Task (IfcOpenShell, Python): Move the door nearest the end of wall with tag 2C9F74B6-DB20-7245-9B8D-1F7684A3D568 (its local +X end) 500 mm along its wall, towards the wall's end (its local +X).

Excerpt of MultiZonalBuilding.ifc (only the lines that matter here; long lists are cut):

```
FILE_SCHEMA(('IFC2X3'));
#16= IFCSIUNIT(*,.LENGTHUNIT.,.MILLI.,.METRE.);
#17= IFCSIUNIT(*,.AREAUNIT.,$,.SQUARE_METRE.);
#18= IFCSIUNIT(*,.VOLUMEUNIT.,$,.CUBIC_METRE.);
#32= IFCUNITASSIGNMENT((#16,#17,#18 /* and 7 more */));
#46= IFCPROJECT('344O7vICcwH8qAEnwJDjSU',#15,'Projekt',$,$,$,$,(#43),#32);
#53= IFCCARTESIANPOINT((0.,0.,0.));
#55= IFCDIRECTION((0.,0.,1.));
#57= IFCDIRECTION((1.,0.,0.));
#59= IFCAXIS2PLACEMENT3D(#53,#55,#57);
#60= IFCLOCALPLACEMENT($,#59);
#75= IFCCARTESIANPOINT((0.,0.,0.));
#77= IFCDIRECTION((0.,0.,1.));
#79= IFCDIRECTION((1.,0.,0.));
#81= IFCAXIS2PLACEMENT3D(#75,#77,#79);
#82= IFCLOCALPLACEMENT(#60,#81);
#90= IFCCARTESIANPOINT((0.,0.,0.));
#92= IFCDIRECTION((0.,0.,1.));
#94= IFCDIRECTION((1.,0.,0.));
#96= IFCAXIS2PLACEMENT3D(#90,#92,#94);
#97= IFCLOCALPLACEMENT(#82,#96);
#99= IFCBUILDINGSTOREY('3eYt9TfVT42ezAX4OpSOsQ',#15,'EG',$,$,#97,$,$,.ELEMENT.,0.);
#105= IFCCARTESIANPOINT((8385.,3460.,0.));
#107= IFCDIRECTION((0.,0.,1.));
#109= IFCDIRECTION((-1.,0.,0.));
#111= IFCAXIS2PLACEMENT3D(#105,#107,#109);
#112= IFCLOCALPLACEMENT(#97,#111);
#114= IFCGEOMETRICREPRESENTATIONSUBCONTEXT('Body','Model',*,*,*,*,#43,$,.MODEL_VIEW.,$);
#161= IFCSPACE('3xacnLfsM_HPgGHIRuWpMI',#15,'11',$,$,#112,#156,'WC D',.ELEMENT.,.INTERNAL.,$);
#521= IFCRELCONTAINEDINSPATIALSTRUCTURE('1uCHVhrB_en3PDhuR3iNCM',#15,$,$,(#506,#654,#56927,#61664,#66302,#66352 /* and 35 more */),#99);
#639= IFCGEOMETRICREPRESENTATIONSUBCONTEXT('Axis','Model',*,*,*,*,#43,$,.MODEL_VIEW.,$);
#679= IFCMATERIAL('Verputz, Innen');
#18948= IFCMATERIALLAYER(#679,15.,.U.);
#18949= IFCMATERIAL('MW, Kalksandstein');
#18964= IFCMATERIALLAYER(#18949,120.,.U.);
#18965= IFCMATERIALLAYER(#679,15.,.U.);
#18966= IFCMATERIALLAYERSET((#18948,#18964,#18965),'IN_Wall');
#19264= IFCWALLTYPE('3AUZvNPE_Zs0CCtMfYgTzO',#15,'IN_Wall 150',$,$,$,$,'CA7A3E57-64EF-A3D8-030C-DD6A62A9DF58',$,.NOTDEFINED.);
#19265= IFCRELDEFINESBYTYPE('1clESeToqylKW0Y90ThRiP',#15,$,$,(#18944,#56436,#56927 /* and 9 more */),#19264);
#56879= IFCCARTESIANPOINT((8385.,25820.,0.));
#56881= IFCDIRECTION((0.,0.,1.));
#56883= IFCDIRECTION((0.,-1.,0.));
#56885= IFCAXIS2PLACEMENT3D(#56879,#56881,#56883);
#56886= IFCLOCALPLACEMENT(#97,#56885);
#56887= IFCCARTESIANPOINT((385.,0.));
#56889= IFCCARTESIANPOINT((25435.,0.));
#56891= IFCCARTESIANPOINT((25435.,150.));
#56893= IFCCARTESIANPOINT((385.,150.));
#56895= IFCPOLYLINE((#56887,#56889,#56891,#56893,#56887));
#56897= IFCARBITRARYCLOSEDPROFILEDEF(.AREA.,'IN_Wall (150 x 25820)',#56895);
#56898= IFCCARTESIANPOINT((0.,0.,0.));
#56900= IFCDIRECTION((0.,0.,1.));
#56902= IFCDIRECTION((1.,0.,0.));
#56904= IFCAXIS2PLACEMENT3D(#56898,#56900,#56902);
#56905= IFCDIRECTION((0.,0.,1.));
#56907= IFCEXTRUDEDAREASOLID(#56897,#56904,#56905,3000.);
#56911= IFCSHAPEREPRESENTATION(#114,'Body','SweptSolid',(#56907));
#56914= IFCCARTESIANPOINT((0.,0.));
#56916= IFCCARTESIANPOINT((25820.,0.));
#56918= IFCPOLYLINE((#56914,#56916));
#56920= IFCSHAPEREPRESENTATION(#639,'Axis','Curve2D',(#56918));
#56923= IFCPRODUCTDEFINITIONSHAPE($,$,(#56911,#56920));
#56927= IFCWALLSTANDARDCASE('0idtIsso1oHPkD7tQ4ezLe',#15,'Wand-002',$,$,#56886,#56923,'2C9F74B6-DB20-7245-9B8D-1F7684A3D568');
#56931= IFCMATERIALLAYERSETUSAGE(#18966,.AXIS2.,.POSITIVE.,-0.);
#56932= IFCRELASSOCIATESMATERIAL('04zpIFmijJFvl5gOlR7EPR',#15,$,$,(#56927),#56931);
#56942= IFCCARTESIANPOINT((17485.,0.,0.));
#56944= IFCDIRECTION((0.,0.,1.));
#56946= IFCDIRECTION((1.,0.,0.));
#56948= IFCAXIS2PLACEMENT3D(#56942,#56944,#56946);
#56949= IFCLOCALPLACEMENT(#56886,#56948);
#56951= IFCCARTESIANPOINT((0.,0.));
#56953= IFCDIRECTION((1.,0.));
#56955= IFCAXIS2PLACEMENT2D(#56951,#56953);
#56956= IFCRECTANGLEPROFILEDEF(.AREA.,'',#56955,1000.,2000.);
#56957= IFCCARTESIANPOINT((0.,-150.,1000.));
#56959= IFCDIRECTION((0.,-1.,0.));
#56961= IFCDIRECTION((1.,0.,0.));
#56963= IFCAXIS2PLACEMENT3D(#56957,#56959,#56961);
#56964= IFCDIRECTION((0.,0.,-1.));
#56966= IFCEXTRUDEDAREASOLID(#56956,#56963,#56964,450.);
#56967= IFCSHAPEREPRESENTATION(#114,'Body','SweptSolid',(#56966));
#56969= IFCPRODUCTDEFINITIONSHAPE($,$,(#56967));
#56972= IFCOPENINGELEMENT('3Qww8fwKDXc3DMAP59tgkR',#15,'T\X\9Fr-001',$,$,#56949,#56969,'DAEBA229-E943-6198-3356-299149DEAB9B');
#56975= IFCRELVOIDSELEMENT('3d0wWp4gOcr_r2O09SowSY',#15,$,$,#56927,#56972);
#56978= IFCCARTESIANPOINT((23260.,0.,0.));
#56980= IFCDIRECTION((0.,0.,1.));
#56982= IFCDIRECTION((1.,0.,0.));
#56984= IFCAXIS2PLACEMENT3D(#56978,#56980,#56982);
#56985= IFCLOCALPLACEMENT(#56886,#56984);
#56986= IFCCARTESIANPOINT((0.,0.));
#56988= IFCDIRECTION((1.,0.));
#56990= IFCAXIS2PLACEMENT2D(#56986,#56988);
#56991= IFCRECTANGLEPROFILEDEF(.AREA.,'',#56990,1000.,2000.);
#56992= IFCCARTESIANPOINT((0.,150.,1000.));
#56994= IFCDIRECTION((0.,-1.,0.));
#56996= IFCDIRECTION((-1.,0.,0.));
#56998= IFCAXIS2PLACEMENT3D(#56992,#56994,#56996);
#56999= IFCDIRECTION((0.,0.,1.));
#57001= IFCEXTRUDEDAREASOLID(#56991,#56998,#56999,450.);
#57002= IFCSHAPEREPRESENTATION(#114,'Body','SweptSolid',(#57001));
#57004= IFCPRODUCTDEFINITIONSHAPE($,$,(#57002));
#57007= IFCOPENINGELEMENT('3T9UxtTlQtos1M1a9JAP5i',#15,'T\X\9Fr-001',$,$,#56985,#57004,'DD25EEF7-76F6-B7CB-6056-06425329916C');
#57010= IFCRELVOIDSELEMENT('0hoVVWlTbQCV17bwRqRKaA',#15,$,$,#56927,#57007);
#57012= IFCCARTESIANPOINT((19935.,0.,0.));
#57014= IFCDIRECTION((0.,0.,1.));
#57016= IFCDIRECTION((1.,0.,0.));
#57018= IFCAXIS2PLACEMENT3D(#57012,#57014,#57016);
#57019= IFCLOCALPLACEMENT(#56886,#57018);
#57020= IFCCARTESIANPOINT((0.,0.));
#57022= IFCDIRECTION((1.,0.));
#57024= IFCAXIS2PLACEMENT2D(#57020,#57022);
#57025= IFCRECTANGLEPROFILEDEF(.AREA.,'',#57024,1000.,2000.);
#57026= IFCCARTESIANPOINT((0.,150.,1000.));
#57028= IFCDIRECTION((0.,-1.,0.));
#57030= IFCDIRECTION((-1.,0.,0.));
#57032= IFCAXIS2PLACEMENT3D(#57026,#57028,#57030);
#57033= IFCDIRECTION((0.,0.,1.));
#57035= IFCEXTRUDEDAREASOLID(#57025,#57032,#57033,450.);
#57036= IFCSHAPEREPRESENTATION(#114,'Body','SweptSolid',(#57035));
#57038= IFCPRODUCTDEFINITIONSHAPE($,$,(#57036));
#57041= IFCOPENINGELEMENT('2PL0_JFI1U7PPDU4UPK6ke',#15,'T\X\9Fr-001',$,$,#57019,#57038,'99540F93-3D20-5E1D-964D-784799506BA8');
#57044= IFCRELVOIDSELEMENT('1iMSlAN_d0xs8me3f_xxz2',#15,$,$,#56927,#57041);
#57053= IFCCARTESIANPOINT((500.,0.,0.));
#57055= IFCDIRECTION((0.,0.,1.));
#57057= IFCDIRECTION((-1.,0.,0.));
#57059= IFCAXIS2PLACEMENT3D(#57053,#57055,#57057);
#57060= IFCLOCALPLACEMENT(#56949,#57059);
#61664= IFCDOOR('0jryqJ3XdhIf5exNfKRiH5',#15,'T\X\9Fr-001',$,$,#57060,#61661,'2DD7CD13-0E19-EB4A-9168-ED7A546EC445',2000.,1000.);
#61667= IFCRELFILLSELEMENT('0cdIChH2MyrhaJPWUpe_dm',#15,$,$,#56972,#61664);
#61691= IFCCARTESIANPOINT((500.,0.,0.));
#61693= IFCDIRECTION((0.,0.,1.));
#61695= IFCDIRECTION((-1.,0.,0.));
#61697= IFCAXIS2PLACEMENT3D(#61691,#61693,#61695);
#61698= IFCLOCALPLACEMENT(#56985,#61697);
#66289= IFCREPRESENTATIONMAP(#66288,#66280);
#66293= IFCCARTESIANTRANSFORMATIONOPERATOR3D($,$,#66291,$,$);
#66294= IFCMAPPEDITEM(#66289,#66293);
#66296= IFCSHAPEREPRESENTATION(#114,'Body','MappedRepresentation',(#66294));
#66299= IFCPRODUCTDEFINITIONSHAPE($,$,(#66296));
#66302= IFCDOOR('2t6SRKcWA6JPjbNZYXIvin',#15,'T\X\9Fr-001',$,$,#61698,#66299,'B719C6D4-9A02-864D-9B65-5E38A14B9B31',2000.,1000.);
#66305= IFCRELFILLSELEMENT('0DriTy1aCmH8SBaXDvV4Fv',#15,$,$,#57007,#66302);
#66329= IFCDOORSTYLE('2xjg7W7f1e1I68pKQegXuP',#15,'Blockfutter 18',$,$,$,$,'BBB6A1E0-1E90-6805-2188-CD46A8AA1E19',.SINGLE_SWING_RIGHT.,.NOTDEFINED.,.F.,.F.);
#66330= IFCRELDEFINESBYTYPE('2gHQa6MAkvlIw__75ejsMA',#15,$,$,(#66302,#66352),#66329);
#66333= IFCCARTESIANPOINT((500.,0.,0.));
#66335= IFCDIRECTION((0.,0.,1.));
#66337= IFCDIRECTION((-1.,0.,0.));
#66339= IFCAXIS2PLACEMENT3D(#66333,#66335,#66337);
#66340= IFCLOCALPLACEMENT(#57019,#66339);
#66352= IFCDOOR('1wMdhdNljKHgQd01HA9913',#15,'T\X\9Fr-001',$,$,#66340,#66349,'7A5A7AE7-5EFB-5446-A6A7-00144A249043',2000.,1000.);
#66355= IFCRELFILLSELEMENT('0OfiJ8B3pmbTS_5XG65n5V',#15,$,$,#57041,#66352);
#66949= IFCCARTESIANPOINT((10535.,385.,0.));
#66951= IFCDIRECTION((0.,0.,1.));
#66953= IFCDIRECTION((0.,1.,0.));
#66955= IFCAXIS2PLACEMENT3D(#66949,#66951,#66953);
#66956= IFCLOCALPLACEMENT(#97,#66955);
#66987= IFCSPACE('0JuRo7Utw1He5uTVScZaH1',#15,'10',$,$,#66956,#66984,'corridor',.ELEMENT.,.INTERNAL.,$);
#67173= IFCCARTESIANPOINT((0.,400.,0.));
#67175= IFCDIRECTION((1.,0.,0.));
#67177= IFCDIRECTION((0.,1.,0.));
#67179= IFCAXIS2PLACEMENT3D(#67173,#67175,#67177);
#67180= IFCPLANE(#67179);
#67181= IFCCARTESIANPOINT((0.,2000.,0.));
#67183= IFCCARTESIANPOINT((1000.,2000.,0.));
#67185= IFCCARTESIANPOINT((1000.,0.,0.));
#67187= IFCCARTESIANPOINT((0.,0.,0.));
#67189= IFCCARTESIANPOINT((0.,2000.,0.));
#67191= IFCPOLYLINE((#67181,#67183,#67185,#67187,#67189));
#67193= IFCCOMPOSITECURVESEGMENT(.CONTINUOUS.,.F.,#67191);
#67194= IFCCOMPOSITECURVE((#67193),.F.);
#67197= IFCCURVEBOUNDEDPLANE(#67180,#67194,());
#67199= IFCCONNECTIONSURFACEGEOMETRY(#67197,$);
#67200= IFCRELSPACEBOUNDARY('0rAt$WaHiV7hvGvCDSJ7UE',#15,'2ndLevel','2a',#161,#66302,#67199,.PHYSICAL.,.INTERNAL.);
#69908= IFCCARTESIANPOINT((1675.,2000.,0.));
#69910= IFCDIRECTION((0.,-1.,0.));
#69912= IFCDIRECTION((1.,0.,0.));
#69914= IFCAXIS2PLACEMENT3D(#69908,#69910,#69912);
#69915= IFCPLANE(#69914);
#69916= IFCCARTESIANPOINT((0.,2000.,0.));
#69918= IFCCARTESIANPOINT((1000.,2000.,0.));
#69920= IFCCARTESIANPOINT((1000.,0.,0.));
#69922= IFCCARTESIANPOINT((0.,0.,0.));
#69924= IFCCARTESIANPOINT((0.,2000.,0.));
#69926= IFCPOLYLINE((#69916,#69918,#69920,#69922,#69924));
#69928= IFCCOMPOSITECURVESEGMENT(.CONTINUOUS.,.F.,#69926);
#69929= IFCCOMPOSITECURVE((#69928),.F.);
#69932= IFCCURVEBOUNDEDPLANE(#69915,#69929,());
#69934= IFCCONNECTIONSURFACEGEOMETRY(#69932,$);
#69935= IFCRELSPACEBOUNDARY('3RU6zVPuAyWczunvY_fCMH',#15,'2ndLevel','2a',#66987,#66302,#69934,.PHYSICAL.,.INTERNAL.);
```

```python
import numpy as np
import ifcopenshell
import ifcopenshell.api.geometry
import ifcopenshell.util.placement

model = ifcopenshell.open("MultiZonalBuilding.ifc")

door = model.by_guid("2t6SRKcWA6JPjbNZYXIvin")
opening = door.FillsVoids[0].RelatingOpeningElement
wall = opening.VoidsElements[0].RelatingBuildingElement

wall_matrix = ifcopenshell.util.placement.get_local_placement(wall.ObjectPlacement)
shift = wall_matrix[:3, 0] * 500.0
before = ifcopenshell.util.placement.get_local_placement(door.ObjectPlacement)[:3, 3].copy()

# The door is placed relative to its opening, so it follows when the opening moves.
matrix = ifcopenshell.util.placement.get_local_placement(opening.ObjectPlacement)
matrix[:3, 3] += shift
ifcopenshell.api.geometry.edit_object_placement(
    model, product=opening, matrix=matrix, is_si=False, should_transform_children=True
)

# Space boundary surfaces are stored in each space's coordinates; move them too.
for rel in door.ProvidesBoundaries:
    if not rel.ConnectionGeometry:
        continue
    surface = rel.ConnectionGeometry.SurfaceOnRelatingElement.BasisSurface
    space_matrix = ifcopenshell.util.placement.get_local_placement(rel.RelatingSpace.ObjectPlacement)
    point = np.array(surface.Position.Location.Coordinates) + space_matrix[:3, :3].T @ shift
    surface.Position = model.createIfcAxis2Placement3D(
        model.createIfcCartesianPoint(point.tolist()), surface.Position.Axis, surface.Position.RefDirection
    )

after = ifcopenshell.util.placement.get_local_placement(door.ObjectPlacement)[:3, 3]
print("door moved by", (after - before).round(3) + 0.0)

model.write("MultiZonalBuilding_rev.ifc")
```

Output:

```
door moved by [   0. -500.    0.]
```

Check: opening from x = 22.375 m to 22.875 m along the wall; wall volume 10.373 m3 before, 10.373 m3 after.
